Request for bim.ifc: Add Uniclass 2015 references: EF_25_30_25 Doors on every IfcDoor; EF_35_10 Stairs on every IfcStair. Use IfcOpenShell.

First a look at what the model holds.

```python
import ifcopenshell

model = ifcopenshell.open("bim.ifc")
print(model.schema)
print("classifications:", [c.Name for c in model.by_type("IfcClassification")])
for ifc_class in ("IfcDoor", "IfcRoof", "IfcStair", "IfcWall", "IfcWindow"):
    print(ifc_class, len(model.by_type(ifc_class)))
```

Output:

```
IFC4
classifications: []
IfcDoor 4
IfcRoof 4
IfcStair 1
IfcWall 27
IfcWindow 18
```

```python
import ifcopenshell
import ifcopenshell.api.classification

model = ifcopenshell.open("bim.ifc")

system = ifcopenshell.api.classification.add_classification(model, classification="Uniclass 2015")

codes = {
    "IfcDoor": ("EF_25_30_25", "Doors"),
    "IfcStair": ("EF_35_10", "Stairs"),
}
for ifc_class, (code, name) in codes.items():
    products = model.by_type(ifc_class)
    ifcopenshell.api.classification.add_reference(
        model, products=products, classification=system, identification=code, name=name
    )
    print(code, len(products))

model.write("bim_v2.ifc")
```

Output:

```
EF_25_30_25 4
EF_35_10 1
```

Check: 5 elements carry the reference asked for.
